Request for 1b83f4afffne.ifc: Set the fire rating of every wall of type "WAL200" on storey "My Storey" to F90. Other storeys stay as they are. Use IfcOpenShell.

First a look at what the model holds.

```python
import ifcopenshell
import ifcopenshell.util.element

model = ifcopenshell.open("1b83f4afffne.ifc")
print(model.schema)
storey = next(s for s in model.by_type("IfcBuildingStorey") if s.Name == "My Storey")
walls = [e for e in ifcopenshell.util.element.get_decomposition(storey) if e.is_a("IfcWall")]
seen = {}
for e in walls:
    element_type = ifcopenshell.util.element.get_type(e)
    key = (element_type.Name if element_type != e and element_type else None, ifcopenshell.util.element.get_pset(e, "Pset_WallCommon", "FireRating"))
    seen[key] = seen.get(key, 0) + 1
for (name, value), count in sorted(seen.items(), key=str):
    print(count, "x", name, "|", value)
```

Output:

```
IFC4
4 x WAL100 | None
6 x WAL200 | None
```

```python
import ifcopenshell
import ifcopenshell.api.pset
import ifcopenshell.util.element

model = ifcopenshell.open("1b83f4afffne.ifc")

storey = next(s for s in model.by_type("IfcBuildingStorey") if s.Name == "My Storey")
walls = [e for e in ifcopenshell.util.element.get_decomposition(storey) if e.is_a("IfcWall")]

count = 0
for e in walls:
    element_type = ifcopenshell.util.element.get_type(e)
    if element_type in (None, e) or element_type.Name != "WAL200":
        continue
    # add_pset returns the element's existing set when there is one.
    pset = ifcopenshell.api.pset.add_pset(model, product=e, name="Pset_WallCommon")
    ifcopenshell.api.pset.edit_pset(model, pset=pset, properties={"FireRating": "F90"})
    count += 1

print(count, "walls updated")

model.write("1b83f4afffne_edited.ifc")
```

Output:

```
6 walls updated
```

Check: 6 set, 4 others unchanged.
